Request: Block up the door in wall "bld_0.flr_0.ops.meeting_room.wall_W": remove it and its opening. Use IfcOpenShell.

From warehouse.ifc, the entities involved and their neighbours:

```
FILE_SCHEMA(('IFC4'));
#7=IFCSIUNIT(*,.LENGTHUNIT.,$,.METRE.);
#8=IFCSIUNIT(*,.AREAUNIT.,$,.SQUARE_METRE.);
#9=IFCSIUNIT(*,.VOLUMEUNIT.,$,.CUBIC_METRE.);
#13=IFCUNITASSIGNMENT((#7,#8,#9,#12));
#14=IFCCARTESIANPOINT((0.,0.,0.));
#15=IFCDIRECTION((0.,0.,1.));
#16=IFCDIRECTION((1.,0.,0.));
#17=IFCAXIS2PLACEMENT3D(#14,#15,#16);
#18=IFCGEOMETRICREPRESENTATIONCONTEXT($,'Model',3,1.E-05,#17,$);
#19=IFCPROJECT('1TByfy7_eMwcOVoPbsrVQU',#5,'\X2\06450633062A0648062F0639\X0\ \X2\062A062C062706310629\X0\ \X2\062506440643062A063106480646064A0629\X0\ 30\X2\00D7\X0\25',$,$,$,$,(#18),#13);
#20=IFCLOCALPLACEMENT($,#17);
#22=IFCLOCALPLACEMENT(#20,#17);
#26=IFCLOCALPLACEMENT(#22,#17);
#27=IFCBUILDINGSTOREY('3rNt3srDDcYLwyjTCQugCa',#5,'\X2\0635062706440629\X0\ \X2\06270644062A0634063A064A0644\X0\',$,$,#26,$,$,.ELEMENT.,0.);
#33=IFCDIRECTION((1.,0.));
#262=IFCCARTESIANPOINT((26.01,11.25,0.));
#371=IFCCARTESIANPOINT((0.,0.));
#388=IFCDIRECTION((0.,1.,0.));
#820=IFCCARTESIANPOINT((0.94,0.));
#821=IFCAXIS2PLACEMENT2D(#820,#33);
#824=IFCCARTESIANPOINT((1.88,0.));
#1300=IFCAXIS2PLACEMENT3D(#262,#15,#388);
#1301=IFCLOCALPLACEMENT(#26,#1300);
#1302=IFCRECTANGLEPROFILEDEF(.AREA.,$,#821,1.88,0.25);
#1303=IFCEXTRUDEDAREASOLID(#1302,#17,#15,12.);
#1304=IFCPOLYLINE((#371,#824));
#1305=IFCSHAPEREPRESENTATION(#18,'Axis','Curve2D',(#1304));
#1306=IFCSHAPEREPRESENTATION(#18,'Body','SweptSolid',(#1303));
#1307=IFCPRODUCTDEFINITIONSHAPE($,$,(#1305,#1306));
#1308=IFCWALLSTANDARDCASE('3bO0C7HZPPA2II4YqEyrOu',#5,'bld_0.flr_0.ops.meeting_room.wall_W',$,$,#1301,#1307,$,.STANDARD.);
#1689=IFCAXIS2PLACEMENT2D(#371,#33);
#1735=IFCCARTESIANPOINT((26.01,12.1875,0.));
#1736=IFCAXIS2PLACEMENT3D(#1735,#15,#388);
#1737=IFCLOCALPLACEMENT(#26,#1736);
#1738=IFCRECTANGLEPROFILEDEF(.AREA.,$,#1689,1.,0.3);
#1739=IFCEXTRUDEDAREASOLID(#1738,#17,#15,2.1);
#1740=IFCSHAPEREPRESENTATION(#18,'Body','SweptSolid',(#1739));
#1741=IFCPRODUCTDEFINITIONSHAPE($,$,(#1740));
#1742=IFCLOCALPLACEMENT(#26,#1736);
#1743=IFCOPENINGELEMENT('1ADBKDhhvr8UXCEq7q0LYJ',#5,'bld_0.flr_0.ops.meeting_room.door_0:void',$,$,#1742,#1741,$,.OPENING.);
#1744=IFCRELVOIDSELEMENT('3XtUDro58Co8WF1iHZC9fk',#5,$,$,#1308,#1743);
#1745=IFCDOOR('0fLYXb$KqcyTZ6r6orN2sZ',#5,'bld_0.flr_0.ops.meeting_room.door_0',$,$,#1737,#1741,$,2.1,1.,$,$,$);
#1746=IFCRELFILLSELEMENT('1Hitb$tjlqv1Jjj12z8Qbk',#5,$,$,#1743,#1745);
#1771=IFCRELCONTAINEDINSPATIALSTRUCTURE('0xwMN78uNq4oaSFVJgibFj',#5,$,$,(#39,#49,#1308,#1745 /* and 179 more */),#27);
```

```python
import ifcopenshell
import ifcopenshell.api.feature
import ifcopenshell.api.root
import ifcopenshell.geom
import ifcopenshell.util.shape

model = ifcopenshell.open("warehouse.ifc")
settings = ifcopenshell.geom.settings()


def volume(element):
    """Net volume in cubic metres, openings subtracted."""
    shape = ifcopenshell.geom.create_shape(settings, element)
    return ifcopenshell.util.shape.get_volume(shape.geometry)


door = model.by_id(1745)
opening = door.FillsVoids[0].RelatingOpeningElement
wall = opening.VoidsElements[0].RelatingBuildingElement
before = volume(wall)

ifcopenshell.api.root.remove_product(model, product=door)
ifcopenshell.api.feature.remove_feature(model, feature=opening)

after = volume(wall)

print(f"wall volume {before:.3f} -> {after:.3f} m3")

model.write("warehouse_edited.ifc")
```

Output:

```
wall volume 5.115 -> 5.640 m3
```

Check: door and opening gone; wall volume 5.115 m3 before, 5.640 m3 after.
